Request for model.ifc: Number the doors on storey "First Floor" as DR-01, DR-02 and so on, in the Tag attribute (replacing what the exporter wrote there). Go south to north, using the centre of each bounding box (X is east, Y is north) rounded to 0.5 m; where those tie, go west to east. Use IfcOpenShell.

First a look at what the model holds.

```python
import ifcopenshell
import ifcopenshell.util.element
import ifcopenshell.util.placement

model = ifcopenshell.open("model.ifc")
print(model.schema)
storey = next(s for s in model.by_type("IfcBuildingStorey") if s.Name == "First Floor")
doors = [e for e in ifcopenshell.util.element.get_decomposition(storey) if e.is_a("IfcDoor")]
for e in sorted(doors, key=lambda e: e.id()):
    origin = ifcopenshell.util.placement.get_local_placement(e.ObjectPlacement)[:3, 3]
    print(e.id(), e.Tag, e.Name, origin.round(2) + 0.0, sep=" | ")
```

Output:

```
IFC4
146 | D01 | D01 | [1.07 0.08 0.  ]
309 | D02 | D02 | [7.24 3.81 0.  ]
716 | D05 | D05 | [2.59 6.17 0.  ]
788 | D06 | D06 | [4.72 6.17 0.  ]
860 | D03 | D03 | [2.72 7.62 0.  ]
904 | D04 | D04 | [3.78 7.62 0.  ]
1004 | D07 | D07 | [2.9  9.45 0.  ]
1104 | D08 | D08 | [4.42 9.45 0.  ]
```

```python
import ifcopenshell
import ifcopenshell.geom
import ifcopenshell.util.element
import ifcopenshell.util.shape

model = ifcopenshell.open("model.ifc")
settings = ifcopenshell.geom.settings()
settings.set("use-world-coords", True)


def centre(element):
    shape = ifcopenshell.geom.create_shape(settings, element)
    return ifcopenshell.util.shape.get_bbox_centroid(shape.geometry)


storey = next(s for s in model.by_type("IfcBuildingStorey") if s.Name == "First Floor")
doors = [e for e in ifcopenshell.util.element.get_decomposition(storey) if e.is_a("IfcDoor")]

# Insertion points can sit at a corner or the storey origin, so sort by the geometry (in metres).
centres = {e: centre(e) for e in doors}
doors.sort(key=lambda e: (round(centres[e][1] / 0.5), centres[e][0]))

for i, e in enumerate(doors, start=1):
    number = f"DR-{i:02d}"
    e.Tag = number
    print(e.id(), number)

model.write("model_rev.ifc")
```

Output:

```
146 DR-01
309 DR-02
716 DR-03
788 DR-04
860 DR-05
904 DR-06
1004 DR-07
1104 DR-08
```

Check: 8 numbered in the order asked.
